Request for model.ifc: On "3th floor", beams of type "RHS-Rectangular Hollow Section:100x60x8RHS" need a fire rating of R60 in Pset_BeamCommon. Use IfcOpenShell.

First a look at what the model holds.

```python
import ifcopenshell
import ifcopenshell.util.element

model = ifcopenshell.open("model.ifc")
print(model.schema)
storey = next(s for s in model.by_type("IfcBuildingStorey") if s.Name == "3th floor")
beams = [e for e in ifcopenshell.util.element.get_decomposition(storey) if e.is_a("IfcBeam")]
seen = {}
for e in beams:
    element_type = ifcopenshell.util.element.get_type(e)
    key = (element_type.Name if element_type != e and element_type else None, ifcopenshell.util.element.get_pset(e, "Pset_BeamCommon", "FireRating"))
    seen[key] = seen.get(key, 0) + 1
for (name, value), count in sorted(seen.items(), key=str):
    print(count, "x", name, "|", value)
```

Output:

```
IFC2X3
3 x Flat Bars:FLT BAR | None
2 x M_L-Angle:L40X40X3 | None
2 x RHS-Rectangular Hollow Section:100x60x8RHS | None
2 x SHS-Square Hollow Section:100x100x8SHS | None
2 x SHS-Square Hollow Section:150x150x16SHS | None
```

```python
import ifcopenshell
import ifcopenshell.api.pset
import ifcopenshell.util.element

model = ifcopenshell.open("model.ifc")

storey = next(s for s in model.by_type("IfcBuildingStorey") if s.Name == "3th floor")
beams = [e for e in ifcopenshell.util.element.get_decomposition(storey) if e.is_a("IfcBeam")]

count = 0
for e in beams:
    element_type = ifcopenshell.util.element.get_type(e)
    if element_type in (None, e) or element_type.Name != "RHS-Rectangular Hollow Section:100x60x8RHS":
        continue
    # add_pset returns the element's existing set when there is one.
    pset = ifcopenshell.api.pset.add_pset(model, product=e, name="Pset_BeamCommon")
    ifcopenshell.api.pset.edit_pset(model, pset=pset, properties={"FireRating": "R60"})
    count += 1

print(count, "beams updated")

model.write("model_rev.ifc")
```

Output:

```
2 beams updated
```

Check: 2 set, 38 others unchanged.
